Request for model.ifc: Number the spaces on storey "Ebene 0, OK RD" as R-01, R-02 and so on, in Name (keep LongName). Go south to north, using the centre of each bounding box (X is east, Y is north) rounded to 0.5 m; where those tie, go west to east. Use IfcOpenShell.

First a look at what the model holds.

```python
import ifcopenshell
import ifcopenshell.util.element
import ifcopenshell.util.placement

model = ifcopenshell.open("model.ifc")
print(model.schema)
storey = next(s for s in model.by_type("IfcBuildingStorey") if s.Name == "Ebene 0, OK RD")
spaces = [e for e in ifcopenshell.util.element.get_decomposition(storey) if e.is_a("IfcSpace")]
for e in sorted(spaces, key=lambda e: e.id()):
    origin = ifcopenshell.util.placement.get_local_placement(e.ObjectPlacement)[:3, 3]
    print(e.id(), e.Name, e.LongName, origin.round(2) + 0.0, sep=" | ")
```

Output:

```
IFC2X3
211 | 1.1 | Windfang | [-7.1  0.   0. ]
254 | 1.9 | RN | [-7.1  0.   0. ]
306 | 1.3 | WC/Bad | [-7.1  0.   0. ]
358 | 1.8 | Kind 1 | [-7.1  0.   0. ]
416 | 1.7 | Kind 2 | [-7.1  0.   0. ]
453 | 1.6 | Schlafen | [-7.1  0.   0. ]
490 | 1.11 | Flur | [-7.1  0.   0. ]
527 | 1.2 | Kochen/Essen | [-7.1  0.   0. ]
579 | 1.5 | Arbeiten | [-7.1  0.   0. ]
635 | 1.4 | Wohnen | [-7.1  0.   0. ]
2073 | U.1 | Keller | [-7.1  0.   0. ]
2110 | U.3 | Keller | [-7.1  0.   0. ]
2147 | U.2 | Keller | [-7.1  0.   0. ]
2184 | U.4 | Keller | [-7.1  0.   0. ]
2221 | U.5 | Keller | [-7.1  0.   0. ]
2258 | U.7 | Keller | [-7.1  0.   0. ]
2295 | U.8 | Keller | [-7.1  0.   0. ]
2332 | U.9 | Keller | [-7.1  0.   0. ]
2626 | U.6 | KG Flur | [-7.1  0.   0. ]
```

```python
import ifcopenshell
import ifcopenshell.geom
import ifcopenshell.util.element
import ifcopenshell.util.shape

model = ifcopenshell.open("model.ifc")
settings = ifcopenshell.geom.settings()
settings.set("use-world-coords", True)


def centre(element):
    shape = ifcopenshell.geom.create_shape(settings, element)
    return ifcopenshell.util.shape.get_bbox_centroid(shape.geometry)


storey = next(s for s in model.by_type("IfcBuildingStorey") if s.Name == "Ebene 0, OK RD")
spaces = [e for e in ifcopenshell.util.element.get_decomposition(storey) if e.is_a("IfcSpace")]

# Insertion points can sit at a corner or the storey origin, so sort by the geometry (in metres).
centres = {e: centre(e) for e in spaces}
spaces.sort(key=lambda e: (round(centres[e][1] / 0.5), centres[e][0]))

for i, e in enumerate(spaces, start=1):
    number = f"R-{i:02d}"
    e.Name = number
    print(e.id(), number)

model.write("model_rev.ifc")
```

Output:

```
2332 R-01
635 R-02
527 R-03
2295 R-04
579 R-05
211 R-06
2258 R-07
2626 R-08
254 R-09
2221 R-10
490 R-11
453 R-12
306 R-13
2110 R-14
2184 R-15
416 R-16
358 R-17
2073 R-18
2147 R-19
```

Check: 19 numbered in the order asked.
